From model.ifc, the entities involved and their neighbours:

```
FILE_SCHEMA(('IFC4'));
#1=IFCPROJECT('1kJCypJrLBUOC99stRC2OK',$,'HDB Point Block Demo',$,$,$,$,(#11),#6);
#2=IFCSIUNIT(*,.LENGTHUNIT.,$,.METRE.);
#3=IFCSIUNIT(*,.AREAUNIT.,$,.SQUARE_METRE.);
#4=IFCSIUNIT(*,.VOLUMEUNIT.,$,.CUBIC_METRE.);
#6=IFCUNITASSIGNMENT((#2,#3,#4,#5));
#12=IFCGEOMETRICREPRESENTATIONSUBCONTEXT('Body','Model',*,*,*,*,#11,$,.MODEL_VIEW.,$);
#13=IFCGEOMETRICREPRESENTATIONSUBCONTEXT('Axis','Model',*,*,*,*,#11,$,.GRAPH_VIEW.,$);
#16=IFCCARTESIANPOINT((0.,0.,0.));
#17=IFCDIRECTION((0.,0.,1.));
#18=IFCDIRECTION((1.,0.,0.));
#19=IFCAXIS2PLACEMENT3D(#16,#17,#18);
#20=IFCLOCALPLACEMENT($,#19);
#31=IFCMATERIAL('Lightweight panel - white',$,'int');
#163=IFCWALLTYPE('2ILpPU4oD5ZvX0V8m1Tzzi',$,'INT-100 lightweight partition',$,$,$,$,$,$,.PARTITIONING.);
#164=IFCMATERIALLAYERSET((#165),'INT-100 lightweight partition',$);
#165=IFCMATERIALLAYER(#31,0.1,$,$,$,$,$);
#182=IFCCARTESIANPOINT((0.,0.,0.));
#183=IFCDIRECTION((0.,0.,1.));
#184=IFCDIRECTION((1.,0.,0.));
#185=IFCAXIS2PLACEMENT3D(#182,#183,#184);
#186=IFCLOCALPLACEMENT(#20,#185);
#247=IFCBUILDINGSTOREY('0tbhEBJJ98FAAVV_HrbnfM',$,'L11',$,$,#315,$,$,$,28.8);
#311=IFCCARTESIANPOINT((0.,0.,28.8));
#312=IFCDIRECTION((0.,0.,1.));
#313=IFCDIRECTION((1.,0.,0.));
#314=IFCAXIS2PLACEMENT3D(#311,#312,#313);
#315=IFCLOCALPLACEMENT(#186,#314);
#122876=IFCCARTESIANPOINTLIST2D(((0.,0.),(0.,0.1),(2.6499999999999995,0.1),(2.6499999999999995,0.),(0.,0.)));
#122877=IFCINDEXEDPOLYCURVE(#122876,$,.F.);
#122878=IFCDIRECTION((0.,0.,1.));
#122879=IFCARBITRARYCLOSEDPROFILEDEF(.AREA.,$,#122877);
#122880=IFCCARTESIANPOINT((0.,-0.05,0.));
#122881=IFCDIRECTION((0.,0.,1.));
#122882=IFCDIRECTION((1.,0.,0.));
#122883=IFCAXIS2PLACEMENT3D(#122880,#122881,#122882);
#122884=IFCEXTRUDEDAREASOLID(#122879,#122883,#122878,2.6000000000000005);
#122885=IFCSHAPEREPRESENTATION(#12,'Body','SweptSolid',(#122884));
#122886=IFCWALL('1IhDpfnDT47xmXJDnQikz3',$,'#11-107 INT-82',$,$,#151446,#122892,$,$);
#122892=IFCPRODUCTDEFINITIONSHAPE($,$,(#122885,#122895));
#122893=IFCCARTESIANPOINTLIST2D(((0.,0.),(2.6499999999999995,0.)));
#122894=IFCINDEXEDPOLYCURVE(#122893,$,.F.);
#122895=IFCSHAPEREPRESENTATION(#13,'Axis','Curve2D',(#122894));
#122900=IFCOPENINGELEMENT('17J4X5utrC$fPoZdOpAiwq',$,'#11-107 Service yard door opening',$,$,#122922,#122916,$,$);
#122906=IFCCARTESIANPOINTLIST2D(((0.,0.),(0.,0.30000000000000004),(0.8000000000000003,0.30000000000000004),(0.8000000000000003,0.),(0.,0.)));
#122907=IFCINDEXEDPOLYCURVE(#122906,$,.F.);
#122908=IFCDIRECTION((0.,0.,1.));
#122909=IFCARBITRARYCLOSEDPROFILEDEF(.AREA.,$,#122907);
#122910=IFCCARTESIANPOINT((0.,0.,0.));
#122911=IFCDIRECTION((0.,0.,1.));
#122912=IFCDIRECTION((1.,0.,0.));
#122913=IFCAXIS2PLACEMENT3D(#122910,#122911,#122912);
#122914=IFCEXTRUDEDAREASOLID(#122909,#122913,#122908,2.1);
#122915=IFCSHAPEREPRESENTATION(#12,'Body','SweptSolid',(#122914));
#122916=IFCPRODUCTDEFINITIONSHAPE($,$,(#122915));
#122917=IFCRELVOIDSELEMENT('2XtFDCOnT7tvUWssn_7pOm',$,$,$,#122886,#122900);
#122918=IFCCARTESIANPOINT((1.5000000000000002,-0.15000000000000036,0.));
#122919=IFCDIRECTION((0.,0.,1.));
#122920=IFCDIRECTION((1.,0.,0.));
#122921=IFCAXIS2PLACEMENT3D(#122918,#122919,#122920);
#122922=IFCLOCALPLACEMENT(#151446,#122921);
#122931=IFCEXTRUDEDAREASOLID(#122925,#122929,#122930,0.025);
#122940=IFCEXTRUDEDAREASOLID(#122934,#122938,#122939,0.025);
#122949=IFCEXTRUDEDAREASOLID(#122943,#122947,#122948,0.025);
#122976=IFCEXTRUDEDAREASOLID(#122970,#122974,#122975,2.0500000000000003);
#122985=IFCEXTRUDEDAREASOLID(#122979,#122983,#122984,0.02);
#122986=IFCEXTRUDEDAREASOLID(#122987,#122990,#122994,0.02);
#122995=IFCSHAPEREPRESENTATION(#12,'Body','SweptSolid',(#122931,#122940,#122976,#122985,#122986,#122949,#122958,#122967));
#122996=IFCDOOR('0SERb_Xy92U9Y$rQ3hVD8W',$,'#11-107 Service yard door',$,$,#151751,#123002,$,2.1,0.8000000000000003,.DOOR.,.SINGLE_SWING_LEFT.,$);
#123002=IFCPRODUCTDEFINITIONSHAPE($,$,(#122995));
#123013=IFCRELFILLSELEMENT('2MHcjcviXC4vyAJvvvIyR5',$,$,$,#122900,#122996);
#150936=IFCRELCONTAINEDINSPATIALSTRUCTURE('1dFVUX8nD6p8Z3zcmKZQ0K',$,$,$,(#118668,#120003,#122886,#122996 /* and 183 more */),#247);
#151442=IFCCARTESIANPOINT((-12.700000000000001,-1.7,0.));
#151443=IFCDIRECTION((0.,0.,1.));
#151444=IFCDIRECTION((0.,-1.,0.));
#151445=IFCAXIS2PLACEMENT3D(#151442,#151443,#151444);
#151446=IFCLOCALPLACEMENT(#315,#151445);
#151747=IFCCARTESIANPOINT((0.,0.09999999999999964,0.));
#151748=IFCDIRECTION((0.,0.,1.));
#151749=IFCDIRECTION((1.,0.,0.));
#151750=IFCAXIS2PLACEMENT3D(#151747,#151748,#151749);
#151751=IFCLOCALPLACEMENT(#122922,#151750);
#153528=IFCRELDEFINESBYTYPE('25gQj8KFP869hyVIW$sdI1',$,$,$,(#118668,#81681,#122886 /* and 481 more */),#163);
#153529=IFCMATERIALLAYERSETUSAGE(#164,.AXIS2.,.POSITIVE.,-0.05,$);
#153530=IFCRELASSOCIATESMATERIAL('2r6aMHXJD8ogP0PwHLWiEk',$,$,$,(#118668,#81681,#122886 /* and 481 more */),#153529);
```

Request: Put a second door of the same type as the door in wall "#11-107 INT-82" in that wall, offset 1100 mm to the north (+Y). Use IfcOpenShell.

```python
import ifcopenshell
import ifcopenshell.api.feature
import ifcopenshell.api.geometry
import ifcopenshell.api.root
import ifcopenshell.geom
import ifcopenshell.util.element
import ifcopenshell.util.placement
import ifcopenshell.util.shape
import ifcopenshell.util.unit

model = ifcopenshell.open("model.ifc")
unit_scale = ifcopenshell.util.unit.calculate_unit_scale(model)
settings = ifcopenshell.geom.settings()


def volume(element):
    """Net volume in cubic metres, openings subtracted."""
    shape = ifcopenshell.geom.create_shape(settings, element)
    return ifcopenshell.util.shape.get_volume(shape.geometry)


door = model.by_guid("0SERb_Xy92U9Y$rQ3hVD8W")
opening = door.FillsVoids[0].RelatingOpeningElement
wall = opening.VoidsElements[0].RelatingBuildingElement
before = volume(wall)
shift = ifcopenshell.util.placement.get_local_placement(wall.ObjectPlacement)[:3, 0] * -1.1 / unit_scale

# copy_class copies the void relationship, type, container and properties, but no geometry.
new_opening = ifcopenshell.api.root.copy_class(model, product=opening)
new_opening.Representation = ifcopenshell.util.element.copy_deep(
    model, opening.Representation, exclude=["IfcGeometricRepresentationContext", "IfcRepresentationMap"]
)
new_door = ifcopenshell.api.root.copy_class(model, product=door)
new_door.Representation = ifcopenshell.util.element.copy_deep(
    model, door.Representation, exclude=["IfcGeometricRepresentationContext", "IfcRepresentationMap"]
)
ifcopenshell.api.feature.add_filling(model, opening=new_opening, element=new_door)

for old, new in ((opening, new_opening), (door, new_door)):
    matrix = ifcopenshell.util.placement.get_local_placement(old.ObjectPlacement)
    matrix[:3, 3] += shift
    ifcopenshell.api.geometry.edit_object_placement(model, product=new, matrix=matrix, is_si=False)

after = volume(wall)

print(f"wall volume {before:.3f} -> {after:.3f} m3")

model.write("model_v2.ifc")
```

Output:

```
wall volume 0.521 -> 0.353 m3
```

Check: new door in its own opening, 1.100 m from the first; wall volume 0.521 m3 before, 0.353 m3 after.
